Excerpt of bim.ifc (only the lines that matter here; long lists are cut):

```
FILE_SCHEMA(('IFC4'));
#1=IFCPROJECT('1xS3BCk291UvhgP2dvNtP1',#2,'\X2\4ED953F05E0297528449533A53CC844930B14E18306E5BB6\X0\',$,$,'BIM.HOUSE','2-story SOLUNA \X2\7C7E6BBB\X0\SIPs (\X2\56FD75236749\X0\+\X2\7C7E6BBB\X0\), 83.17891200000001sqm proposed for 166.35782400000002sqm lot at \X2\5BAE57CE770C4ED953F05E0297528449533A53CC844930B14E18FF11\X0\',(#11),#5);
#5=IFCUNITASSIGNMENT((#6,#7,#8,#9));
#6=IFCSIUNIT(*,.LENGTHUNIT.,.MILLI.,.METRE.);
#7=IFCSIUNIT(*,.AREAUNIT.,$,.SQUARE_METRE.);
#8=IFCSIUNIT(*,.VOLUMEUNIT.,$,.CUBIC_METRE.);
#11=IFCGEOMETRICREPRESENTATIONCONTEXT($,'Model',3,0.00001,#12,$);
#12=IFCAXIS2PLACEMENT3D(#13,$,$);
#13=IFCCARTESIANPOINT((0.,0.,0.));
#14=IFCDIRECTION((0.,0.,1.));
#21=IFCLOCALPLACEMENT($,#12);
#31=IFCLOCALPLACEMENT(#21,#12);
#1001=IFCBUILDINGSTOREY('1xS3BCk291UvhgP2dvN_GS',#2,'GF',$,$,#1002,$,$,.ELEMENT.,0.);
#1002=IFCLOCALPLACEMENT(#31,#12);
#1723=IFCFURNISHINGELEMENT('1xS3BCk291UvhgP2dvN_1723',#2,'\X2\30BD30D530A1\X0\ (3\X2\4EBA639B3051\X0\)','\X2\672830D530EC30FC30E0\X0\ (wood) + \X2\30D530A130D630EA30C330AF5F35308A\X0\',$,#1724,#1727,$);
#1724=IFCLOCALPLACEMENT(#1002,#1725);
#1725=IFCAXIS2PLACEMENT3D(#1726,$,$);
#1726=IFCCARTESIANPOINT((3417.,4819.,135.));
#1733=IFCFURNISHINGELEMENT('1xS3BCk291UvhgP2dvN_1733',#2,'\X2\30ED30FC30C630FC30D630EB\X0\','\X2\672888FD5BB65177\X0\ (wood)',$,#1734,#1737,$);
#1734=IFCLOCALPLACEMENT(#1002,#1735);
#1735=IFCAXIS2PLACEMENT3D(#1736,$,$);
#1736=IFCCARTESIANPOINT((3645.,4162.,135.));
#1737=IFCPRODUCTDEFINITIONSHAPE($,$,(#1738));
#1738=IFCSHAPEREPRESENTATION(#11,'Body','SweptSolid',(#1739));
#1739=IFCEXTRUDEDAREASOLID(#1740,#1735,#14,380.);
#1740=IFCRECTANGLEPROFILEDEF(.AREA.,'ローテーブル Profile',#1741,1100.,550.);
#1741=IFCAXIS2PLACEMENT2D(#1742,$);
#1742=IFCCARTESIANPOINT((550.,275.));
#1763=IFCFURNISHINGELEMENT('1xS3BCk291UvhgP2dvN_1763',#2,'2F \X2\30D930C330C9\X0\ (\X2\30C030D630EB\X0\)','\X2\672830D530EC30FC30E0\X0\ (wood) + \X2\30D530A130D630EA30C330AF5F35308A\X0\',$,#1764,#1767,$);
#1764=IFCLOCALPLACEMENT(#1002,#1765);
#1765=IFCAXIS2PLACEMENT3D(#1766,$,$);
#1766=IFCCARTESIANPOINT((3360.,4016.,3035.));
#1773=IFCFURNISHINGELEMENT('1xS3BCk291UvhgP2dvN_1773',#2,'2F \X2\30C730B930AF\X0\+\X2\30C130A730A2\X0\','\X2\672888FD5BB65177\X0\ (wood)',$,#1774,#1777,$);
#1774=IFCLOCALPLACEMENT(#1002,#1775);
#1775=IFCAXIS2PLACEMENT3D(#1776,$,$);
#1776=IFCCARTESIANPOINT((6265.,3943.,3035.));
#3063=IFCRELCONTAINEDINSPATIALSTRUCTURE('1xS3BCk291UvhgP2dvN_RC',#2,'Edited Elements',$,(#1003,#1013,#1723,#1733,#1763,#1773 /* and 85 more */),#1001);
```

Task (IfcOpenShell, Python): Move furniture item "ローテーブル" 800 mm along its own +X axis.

```python
import ifcopenshell
import ifcopenshell.api.geometry
import ifcopenshell.util.placement
import ifcopenshell.util.unit

model = ifcopenshell.open("bim.ifc")
unit_scale = ifcopenshell.util.unit.calculate_unit_scale(model)

item = model.by_guid("1xS3BCk291UvhgP2dvN_1733")
matrix = ifcopenshell.util.placement.get_local_placement(item.ObjectPlacement)
matrix[:3, 3] += matrix[:3, 0] * 0.8 / unit_scale
ifcopenshell.api.geometry.edit_object_placement(model, product=item, matrix=matrix, is_si=False)

print(ifcopenshell.util.placement.get_local_placement(item.ObjectPlacement).round(3) + 0.0)

model.write("bim_rev.ifc")
```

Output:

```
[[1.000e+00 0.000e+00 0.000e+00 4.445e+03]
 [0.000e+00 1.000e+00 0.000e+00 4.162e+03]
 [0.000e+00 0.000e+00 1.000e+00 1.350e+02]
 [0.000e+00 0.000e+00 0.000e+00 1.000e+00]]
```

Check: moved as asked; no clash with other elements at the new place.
